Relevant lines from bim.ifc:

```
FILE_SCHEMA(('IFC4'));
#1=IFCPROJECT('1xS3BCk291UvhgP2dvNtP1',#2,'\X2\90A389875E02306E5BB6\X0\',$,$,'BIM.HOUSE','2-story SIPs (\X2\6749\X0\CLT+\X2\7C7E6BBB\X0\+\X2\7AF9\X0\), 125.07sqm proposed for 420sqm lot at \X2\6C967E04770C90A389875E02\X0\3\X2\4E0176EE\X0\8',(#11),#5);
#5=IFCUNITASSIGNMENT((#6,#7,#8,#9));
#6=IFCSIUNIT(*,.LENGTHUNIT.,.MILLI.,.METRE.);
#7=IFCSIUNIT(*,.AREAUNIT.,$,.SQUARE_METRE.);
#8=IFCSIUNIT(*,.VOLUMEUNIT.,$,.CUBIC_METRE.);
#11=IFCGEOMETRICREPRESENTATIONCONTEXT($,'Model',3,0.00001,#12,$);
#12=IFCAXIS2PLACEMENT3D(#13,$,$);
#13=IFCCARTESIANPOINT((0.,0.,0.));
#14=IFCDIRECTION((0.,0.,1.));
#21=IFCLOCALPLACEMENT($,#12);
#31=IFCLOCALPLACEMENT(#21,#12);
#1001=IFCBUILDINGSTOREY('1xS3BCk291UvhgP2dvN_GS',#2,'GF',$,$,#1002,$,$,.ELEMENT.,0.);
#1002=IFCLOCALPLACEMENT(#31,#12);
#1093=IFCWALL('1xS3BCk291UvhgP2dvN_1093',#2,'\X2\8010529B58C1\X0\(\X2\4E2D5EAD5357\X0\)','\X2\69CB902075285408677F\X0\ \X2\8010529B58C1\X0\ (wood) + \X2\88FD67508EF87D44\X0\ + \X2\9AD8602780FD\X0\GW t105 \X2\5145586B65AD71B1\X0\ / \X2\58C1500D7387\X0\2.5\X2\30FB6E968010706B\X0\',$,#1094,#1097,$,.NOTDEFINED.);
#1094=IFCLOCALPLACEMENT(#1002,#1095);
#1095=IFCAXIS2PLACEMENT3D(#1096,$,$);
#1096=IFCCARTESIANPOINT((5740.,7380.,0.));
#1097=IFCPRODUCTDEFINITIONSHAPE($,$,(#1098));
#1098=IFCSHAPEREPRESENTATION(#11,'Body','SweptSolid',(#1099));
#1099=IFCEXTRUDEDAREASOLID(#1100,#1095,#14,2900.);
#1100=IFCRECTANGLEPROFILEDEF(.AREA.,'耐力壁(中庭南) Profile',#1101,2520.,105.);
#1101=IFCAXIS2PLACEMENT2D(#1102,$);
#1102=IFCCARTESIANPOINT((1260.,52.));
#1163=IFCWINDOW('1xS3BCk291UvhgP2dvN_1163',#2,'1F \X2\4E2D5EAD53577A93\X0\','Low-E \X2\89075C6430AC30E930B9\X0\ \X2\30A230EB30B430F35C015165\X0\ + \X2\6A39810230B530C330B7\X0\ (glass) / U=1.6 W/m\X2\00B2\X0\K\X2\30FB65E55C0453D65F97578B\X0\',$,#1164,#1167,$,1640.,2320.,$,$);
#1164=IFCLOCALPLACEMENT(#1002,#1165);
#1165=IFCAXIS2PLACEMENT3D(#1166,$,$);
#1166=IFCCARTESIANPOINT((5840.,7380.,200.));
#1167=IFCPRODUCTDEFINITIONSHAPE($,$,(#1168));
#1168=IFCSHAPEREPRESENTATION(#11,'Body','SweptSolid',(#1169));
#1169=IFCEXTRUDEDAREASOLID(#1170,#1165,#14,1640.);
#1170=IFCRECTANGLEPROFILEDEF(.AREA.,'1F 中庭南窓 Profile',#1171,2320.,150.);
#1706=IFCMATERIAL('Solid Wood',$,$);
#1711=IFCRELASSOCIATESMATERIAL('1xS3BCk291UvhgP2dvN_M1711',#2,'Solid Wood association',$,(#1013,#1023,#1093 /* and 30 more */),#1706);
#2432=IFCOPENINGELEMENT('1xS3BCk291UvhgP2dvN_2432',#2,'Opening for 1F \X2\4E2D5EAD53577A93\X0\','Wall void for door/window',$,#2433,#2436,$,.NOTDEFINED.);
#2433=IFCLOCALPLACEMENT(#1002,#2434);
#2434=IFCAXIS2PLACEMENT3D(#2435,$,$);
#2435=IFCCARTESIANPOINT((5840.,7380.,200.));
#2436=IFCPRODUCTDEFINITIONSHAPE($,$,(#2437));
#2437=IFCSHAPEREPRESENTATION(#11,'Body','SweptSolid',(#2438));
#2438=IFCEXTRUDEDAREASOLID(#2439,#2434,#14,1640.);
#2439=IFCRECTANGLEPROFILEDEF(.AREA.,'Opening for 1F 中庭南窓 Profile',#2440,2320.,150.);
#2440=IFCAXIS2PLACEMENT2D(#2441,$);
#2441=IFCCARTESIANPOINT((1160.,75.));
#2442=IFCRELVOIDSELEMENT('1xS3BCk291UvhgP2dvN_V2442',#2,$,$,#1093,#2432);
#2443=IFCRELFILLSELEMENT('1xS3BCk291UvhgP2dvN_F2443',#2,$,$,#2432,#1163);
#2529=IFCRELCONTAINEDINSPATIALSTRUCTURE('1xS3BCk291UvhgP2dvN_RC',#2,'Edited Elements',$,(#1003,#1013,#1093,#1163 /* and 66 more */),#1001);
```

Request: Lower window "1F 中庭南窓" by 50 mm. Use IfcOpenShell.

```python
import numpy as np
import ifcopenshell
import ifcopenshell.api.geometry
import ifcopenshell.util.placement
import ifcopenshell.util.unit

model = ifcopenshell.open("bim.ifc")
unit_scale = ifcopenshell.util.unit.calculate_unit_scale(model)

window = model.by_guid("1xS3BCk291UvhgP2dvN_1163")
opening = window.FillsVoids[0].RelatingOpeningElement
dz = -0.05 / unit_scale

shift = np.array([0.0, 0.0, dz])
# The window is not placed relative to its opening, so move both.
for product in (opening, window):
    matrix = ifcopenshell.util.placement.get_local_placement(product.ObjectPlacement)
    matrix[:3, 3] += shift
    ifcopenshell.api.geometry.edit_object_placement(model, product=product, matrix=matrix, is_si=False)

print(f"moved by {dz * unit_scale:+.3f} m")

model.write("bim_rev.ifc")
```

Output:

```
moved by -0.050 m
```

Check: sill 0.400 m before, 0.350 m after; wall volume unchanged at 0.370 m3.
